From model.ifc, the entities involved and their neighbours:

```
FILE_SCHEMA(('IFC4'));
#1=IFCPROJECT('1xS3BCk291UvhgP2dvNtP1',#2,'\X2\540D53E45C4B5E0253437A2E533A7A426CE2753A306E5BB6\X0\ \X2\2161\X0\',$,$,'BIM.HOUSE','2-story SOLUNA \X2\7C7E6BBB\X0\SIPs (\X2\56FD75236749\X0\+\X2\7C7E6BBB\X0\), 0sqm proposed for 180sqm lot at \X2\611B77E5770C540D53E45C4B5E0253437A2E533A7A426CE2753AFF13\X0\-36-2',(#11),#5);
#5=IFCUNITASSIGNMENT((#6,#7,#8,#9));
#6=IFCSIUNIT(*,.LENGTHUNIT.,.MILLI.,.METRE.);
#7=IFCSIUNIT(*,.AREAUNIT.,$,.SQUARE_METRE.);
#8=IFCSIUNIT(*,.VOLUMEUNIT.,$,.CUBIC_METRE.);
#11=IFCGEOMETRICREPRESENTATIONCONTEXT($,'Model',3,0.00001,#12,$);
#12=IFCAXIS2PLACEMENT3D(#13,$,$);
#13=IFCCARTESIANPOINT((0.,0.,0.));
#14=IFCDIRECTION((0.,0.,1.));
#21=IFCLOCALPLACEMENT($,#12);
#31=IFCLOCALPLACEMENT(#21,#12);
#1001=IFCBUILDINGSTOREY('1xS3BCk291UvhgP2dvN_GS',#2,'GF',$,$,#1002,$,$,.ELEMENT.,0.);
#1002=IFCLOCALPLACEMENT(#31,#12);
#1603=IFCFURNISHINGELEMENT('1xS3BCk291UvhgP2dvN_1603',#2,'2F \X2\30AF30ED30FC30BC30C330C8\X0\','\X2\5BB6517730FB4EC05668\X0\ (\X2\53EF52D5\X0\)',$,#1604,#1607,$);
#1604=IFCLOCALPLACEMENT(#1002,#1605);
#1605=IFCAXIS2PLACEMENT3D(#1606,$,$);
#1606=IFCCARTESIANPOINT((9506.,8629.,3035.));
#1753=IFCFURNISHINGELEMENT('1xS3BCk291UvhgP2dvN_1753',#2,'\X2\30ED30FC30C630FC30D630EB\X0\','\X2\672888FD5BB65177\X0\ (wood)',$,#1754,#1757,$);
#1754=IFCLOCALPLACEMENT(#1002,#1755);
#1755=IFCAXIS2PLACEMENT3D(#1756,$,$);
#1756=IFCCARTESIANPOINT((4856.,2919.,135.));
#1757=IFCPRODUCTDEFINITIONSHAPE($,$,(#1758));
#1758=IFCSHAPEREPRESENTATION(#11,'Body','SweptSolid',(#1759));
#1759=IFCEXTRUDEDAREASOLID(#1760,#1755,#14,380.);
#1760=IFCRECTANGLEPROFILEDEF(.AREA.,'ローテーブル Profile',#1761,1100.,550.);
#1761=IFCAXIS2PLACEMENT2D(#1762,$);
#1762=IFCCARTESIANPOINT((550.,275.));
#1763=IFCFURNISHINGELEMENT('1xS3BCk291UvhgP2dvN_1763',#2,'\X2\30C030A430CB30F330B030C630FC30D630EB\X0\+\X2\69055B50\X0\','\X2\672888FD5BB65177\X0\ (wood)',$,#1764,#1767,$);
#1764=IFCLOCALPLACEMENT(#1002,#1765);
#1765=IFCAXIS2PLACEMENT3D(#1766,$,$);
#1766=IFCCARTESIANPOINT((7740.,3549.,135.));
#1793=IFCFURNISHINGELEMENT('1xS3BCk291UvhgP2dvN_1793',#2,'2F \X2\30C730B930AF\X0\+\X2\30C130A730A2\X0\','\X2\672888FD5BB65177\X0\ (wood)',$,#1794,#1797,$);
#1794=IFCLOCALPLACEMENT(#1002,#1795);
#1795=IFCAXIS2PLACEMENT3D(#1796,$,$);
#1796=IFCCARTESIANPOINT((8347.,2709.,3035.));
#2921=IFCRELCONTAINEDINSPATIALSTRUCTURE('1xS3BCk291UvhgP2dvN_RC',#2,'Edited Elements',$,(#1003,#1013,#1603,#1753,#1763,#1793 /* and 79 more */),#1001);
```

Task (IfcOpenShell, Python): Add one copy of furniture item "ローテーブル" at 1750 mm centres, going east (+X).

```python
import numpy as np
import ifcopenshell
import ifcopenshell.api.geometry
import ifcopenshell.api.root
import ifcopenshell.util.element
import ifcopenshell.util.placement
import ifcopenshell.util.unit

model = ifcopenshell.open("model.ifc")
unit_scale = ifcopenshell.util.unit.calculate_unit_scale(model)


def reuse_history(source, copy):
    """copy_class also copies each property set's owner history, people and application; keep the originals."""
    for rel in copy.IsDefinedBy:
        if rel.is_a("IfcRelDefinesByProperties") and (history := rel.RelatingPropertyDefinition.OwnerHistory):
            rel.RelatingPropertyDefinition.OwnerHistory = source.OwnerHistory
            ifcopenshell.util.element.remove_deep2(model, history)


source = model.by_guid("1xS3BCk291UvhgP2dvN_1753")
base = ifcopenshell.util.placement.get_local_placement(source.ObjectPlacement)
step = np.array([1.0, 0.0, 0.0]) * 1.75 / unit_scale

for i in range(1, 2):
    copy = ifcopenshell.api.root.copy_class(model, product=source)
    copy.Representation = ifcopenshell.util.element.copy_deep(
        model, source.Representation, exclude=["IfcGeometricRepresentationContext", "IfcRepresentationMap"]
    )
    reuse_history(source, copy)
    matrix = base.copy()
    matrix[:3, 3] += i * step
    print("added at", matrix[:3, 3].round(3) + 0.0)
    ifcopenshell.api.geometry.edit_object_placement(model, product=copy, matrix=matrix, is_si=False)

model.write("model_v2.ifc")
```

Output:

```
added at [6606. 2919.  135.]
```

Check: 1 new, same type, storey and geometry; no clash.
